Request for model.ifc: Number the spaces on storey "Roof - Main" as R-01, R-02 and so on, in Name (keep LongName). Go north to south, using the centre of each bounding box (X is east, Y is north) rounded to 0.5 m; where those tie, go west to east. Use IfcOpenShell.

First a look at what the model holds.

```python
import ifcopenshell
import ifcopenshell.util.element
import ifcopenshell.util.placement

model = ifcopenshell.open("model.ifc")
print(model.schema)
storey = next(s for s in model.by_type("IfcBuildingStorey") if s.Name == "Roof - Main")
spaces = [e for e in ifcopenshell.util.element.get_decomposition(storey) if e.is_a("IfcSpace")]
for e in sorted(spaces, key=lambda e: e.id()):
    origin = ifcopenshell.util.placement.get_local_placement(e.ObjectPlacement)[:3, 3]
    print(e.id(), e.Name, e.LongName, origin.round(2) + 0.0, sep=" | ")
```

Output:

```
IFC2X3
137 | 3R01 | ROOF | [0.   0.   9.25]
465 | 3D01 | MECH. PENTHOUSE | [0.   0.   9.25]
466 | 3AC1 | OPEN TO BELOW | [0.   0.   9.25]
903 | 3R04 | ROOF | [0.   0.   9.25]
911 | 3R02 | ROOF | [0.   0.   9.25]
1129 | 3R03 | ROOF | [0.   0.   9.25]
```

```python
import ifcopenshell
import ifcopenshell.geom
import ifcopenshell.util.element
import ifcopenshell.util.shape

model = ifcopenshell.open("model.ifc")
settings = ifcopenshell.geom.settings()
settings.set("use-world-coords", True)


def centre(element):
    shape = ifcopenshell.geom.create_shape(settings, element)
    return ifcopenshell.util.shape.get_bbox_centroid(shape.geometry)


storey = next(s for s in model.by_type("IfcBuildingStorey") if s.Name == "Roof - Main")
spaces = [e for e in ifcopenshell.util.element.get_decomposition(storey) if e.is_a("IfcSpace")]

# Insertion points can sit at a corner or the storey origin, so sort by the geometry (in metres).
centres = {e: centre(e) for e in spaces}
spaces.sort(key=lambda e: (-round(centres[e][1] / 0.5), centres[e][0]))

for i, e in enumerate(spaces, start=1):
    number = f"R-{i:02d}"
    e.Name = number
    print(e.id(), number)

model.write("model_rev.ifc")
```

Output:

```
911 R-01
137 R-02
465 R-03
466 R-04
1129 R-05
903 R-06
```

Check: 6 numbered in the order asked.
